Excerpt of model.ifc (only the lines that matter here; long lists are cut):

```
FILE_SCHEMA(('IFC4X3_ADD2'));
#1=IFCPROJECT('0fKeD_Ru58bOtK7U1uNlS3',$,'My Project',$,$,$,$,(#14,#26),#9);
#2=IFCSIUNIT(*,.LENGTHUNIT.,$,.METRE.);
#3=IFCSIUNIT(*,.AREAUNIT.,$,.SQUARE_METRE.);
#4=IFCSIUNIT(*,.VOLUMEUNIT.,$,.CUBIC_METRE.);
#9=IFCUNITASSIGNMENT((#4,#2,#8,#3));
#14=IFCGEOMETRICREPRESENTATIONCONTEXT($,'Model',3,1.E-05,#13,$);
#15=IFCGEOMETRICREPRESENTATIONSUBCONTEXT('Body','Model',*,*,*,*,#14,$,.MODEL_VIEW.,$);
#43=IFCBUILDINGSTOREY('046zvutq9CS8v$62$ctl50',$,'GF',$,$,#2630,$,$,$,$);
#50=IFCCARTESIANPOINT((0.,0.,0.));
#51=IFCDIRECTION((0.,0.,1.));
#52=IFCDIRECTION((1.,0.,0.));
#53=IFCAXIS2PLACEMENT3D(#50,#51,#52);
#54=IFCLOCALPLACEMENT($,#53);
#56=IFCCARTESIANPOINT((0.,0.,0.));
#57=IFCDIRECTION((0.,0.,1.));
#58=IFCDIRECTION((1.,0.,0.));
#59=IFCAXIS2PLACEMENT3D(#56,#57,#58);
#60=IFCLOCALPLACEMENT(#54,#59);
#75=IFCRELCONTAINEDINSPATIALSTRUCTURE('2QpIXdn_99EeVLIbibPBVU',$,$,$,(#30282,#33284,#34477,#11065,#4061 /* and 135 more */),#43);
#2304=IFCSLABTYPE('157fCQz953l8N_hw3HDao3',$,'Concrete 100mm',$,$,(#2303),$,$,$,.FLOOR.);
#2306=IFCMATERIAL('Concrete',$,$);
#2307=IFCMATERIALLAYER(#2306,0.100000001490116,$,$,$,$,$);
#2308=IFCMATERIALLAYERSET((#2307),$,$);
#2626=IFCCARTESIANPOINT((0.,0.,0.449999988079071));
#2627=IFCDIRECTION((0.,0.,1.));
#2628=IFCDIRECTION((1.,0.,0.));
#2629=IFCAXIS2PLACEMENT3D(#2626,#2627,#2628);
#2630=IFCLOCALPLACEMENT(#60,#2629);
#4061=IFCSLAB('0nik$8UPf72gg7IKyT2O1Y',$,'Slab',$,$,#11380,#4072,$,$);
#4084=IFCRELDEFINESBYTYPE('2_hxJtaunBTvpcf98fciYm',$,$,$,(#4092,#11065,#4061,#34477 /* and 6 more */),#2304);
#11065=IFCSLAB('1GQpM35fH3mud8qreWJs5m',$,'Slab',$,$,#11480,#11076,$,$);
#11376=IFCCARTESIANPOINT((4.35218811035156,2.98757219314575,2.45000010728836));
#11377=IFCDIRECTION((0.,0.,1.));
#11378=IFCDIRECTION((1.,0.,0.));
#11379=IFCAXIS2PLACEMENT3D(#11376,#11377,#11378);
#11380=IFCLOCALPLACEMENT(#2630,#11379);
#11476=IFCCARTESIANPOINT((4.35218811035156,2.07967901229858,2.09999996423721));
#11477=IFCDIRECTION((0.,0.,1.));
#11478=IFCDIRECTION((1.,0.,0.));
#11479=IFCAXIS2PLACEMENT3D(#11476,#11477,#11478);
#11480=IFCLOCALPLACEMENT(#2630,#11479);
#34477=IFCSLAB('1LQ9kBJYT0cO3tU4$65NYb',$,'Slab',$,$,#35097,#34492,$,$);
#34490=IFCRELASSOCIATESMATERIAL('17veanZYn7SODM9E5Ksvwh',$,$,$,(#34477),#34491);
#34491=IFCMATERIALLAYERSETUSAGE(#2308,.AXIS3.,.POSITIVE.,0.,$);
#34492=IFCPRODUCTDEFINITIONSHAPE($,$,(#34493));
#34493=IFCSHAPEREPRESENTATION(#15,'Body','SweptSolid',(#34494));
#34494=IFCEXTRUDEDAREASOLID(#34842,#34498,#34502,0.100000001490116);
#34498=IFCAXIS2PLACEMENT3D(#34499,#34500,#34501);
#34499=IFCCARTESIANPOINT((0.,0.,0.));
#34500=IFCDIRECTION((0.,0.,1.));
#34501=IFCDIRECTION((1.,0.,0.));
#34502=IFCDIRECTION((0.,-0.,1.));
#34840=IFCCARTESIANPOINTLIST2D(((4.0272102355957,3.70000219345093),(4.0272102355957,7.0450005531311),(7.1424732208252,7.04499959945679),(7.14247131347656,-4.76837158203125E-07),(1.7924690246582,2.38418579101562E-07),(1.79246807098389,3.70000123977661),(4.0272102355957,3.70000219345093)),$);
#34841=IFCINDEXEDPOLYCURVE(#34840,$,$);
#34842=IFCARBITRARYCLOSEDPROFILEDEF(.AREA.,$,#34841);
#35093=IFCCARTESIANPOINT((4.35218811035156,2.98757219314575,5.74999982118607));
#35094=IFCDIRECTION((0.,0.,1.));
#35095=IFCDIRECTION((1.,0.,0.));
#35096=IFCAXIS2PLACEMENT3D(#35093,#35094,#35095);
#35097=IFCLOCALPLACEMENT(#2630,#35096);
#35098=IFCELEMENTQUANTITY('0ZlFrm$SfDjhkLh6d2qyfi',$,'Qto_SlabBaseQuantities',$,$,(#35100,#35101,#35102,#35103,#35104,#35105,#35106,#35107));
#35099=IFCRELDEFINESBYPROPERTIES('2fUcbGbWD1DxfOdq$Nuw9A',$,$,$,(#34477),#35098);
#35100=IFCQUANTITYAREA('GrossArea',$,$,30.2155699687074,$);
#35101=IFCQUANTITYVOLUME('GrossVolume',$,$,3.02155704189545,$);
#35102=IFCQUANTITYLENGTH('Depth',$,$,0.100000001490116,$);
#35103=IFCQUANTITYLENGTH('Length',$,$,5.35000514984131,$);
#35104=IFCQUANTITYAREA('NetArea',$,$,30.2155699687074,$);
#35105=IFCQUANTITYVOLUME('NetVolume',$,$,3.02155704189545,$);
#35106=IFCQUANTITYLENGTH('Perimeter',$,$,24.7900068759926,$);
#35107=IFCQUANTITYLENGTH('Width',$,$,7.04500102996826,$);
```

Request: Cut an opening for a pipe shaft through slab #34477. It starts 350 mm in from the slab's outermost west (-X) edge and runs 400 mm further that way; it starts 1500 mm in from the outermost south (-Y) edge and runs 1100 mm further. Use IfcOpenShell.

```python
import numpy as np
import ifcopenshell
import ifcopenshell.api.feature
import ifcopenshell.api.geometry
import ifcopenshell.api.pset
import ifcopenshell.api.root
import ifcopenshell.geom
import ifcopenshell.util.element
import ifcopenshell.util.placement
import ifcopenshell.util.representation
import ifcopenshell.util.shape
import ifcopenshell.util.unit

model = ifcopenshell.open("model.ifc")
unit_scale = ifcopenshell.util.unit.calculate_unit_scale(model)
area_scale = ifcopenshell.util.unit.calculate_unit_scale(model, "AREAUNIT")
volume_scale = ifcopenshell.util.unit.calculate_unit_scale(model, "VOLUMEUNIT")
settings = ifcopenshell.geom.settings()


def volume(element):
    """Net volume in cubic metres, openings subtracted."""
    shape = ifcopenshell.geom.create_shape(settings, element)
    return ifcopenshell.util.shape.get_volume(shape.geometry)


slab = model.by_id(34477)
before = volume(slab)

# Extent in the slab's own axes, in metres. The edges named are its -X and -Y sides.
slab_shape = ifcopenshell.geom.create_shape(settings, slab)
vertices = ifcopenshell.util.shape.get_vertices(slab_shape.geometry)
x_min, y_min, bottom = vertices.min(axis=0)
top = vertices[:, 2].max()

opening = ifcopenshell.api.root.create_entity(model, ifc_class="IfcOpeningElement", name="Pipe shaft opening", predefined_type="OPENING")
context = ifcopenshell.util.representation.get_context(model, "Model", "Body", "MODEL_VIEW")
width, depth = 0.4, 1.1
outline = [(0.0, 0.0), (width, 0.0), (width, depth), (0.0, depth), (0.0, 0.0)]
# Overshoot both faces by 50 mm so the cut is clean.
shape = ifcopenshell.api.geometry.add_slab_representation(
    model, context=context, depth=top - bottom + 0.1, polyline=outline
)
ifcopenshell.api.geometry.assign_representation(model, product=opening, representation=shape)

matrix = ifcopenshell.util.placement.get_local_placement(slab.ObjectPlacement)
matrix[:, 3] = matrix @ np.append(np.array([x_min + 0.35, y_min + 1.5, bottom - 0.05]) / unit_scale, 1.0)
ifcopenshell.api.geometry.edit_object_placement(model, product=opening, matrix=matrix, is_si=False)
ifcopenshell.api.feature.add_feature(model, feature=opening, element=slab)

after = volume(slab)

# Update the slab's stored quantities.
qto = model.by_id(ifcopenshell.util.element.get_pset(slab, "Qto_SlabBaseQuantities", should_inherit=False)["id"])
ifcopenshell.api.pset.edit_qto(model, qto=qto, properties={
    "NetArea": after / (top - bottom) / area_scale,
    "NetVolume": after / volume_scale,
})

print(f"slab volume {before:.3f} -> {after:.3f} m3")

model.write("model-out.ifc")
```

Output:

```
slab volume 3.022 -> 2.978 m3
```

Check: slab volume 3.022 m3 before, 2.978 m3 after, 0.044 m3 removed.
